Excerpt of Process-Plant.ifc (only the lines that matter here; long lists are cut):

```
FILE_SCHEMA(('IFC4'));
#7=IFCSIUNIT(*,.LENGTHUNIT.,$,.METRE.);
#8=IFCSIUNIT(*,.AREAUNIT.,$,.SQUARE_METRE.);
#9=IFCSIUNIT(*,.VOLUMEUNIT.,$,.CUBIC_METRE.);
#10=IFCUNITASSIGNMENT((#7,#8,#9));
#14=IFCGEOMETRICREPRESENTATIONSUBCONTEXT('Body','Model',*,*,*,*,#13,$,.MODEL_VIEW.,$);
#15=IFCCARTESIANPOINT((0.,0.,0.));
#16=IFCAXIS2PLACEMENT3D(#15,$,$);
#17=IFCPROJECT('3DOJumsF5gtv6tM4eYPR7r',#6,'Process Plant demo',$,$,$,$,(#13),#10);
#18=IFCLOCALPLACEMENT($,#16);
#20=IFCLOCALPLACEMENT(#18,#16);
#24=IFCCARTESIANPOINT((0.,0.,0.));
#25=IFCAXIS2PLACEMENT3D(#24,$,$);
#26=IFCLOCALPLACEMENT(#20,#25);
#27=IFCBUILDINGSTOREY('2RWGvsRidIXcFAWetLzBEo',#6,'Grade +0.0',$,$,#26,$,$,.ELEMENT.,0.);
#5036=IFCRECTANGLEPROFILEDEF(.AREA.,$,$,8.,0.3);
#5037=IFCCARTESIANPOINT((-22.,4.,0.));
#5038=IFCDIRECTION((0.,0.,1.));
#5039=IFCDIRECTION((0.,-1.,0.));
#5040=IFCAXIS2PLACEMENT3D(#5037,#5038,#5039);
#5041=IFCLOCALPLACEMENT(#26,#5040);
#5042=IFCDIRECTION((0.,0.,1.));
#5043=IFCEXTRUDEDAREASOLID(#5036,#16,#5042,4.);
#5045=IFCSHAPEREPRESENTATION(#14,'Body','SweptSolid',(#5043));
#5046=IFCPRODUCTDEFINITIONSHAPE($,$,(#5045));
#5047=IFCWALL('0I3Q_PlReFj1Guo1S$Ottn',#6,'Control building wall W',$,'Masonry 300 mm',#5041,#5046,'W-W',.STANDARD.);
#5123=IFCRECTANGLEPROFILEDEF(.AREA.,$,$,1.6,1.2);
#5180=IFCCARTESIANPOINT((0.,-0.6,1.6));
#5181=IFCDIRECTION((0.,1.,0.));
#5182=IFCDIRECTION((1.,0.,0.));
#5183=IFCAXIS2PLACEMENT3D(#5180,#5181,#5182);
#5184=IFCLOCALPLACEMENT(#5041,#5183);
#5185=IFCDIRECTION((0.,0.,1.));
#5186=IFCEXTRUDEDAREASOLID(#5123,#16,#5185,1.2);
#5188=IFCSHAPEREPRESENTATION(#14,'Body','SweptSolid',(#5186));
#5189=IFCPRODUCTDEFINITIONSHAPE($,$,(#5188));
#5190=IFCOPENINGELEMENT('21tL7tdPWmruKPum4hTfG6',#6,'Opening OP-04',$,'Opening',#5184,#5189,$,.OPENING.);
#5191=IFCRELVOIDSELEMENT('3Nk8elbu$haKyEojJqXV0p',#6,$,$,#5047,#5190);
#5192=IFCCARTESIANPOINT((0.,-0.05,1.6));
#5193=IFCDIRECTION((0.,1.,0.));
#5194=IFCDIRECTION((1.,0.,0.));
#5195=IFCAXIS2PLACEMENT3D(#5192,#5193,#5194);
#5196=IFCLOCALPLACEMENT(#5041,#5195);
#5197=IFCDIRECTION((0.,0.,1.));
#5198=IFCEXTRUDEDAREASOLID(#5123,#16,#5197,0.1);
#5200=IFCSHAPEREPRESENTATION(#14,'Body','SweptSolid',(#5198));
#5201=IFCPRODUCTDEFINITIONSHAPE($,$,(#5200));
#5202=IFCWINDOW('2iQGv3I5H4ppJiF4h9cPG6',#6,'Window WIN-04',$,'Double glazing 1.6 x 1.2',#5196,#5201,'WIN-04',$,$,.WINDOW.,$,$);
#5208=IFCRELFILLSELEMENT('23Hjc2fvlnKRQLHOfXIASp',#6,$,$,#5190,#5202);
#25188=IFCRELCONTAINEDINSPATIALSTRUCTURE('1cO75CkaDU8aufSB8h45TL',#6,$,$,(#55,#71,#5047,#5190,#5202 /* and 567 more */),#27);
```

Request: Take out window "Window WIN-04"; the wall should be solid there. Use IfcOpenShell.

```python
import ifcopenshell
import ifcopenshell.api.feature
import ifcopenshell.api.root
import ifcopenshell.geom
import ifcopenshell.util.shape

model = ifcopenshell.open("Process-Plant.ifc")
settings = ifcopenshell.geom.settings()


def volume(element):
    """Net volume in cubic metres, openings subtracted."""
    shape = ifcopenshell.geom.create_shape(settings, element)
    return ifcopenshell.util.shape.get_volume(shape.geometry)


window = model.by_guid("2iQGv3I5H4ppJiF4h9cPG6")
opening = window.FillsVoids[0].RelatingOpeningElement
wall = opening.VoidsElements[0].RelatingBuildingElement
before = volume(wall)

ifcopenshell.api.root.remove_product(model, product=window)
ifcopenshell.api.feature.remove_feature(model, feature=opening)

after = volume(wall)

print(f"wall volume {before:.3f} -> {after:.3f} m3")

model.write("Process-Plant_rev.ifc")
```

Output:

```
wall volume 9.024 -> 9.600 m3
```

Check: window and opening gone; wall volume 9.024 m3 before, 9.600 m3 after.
